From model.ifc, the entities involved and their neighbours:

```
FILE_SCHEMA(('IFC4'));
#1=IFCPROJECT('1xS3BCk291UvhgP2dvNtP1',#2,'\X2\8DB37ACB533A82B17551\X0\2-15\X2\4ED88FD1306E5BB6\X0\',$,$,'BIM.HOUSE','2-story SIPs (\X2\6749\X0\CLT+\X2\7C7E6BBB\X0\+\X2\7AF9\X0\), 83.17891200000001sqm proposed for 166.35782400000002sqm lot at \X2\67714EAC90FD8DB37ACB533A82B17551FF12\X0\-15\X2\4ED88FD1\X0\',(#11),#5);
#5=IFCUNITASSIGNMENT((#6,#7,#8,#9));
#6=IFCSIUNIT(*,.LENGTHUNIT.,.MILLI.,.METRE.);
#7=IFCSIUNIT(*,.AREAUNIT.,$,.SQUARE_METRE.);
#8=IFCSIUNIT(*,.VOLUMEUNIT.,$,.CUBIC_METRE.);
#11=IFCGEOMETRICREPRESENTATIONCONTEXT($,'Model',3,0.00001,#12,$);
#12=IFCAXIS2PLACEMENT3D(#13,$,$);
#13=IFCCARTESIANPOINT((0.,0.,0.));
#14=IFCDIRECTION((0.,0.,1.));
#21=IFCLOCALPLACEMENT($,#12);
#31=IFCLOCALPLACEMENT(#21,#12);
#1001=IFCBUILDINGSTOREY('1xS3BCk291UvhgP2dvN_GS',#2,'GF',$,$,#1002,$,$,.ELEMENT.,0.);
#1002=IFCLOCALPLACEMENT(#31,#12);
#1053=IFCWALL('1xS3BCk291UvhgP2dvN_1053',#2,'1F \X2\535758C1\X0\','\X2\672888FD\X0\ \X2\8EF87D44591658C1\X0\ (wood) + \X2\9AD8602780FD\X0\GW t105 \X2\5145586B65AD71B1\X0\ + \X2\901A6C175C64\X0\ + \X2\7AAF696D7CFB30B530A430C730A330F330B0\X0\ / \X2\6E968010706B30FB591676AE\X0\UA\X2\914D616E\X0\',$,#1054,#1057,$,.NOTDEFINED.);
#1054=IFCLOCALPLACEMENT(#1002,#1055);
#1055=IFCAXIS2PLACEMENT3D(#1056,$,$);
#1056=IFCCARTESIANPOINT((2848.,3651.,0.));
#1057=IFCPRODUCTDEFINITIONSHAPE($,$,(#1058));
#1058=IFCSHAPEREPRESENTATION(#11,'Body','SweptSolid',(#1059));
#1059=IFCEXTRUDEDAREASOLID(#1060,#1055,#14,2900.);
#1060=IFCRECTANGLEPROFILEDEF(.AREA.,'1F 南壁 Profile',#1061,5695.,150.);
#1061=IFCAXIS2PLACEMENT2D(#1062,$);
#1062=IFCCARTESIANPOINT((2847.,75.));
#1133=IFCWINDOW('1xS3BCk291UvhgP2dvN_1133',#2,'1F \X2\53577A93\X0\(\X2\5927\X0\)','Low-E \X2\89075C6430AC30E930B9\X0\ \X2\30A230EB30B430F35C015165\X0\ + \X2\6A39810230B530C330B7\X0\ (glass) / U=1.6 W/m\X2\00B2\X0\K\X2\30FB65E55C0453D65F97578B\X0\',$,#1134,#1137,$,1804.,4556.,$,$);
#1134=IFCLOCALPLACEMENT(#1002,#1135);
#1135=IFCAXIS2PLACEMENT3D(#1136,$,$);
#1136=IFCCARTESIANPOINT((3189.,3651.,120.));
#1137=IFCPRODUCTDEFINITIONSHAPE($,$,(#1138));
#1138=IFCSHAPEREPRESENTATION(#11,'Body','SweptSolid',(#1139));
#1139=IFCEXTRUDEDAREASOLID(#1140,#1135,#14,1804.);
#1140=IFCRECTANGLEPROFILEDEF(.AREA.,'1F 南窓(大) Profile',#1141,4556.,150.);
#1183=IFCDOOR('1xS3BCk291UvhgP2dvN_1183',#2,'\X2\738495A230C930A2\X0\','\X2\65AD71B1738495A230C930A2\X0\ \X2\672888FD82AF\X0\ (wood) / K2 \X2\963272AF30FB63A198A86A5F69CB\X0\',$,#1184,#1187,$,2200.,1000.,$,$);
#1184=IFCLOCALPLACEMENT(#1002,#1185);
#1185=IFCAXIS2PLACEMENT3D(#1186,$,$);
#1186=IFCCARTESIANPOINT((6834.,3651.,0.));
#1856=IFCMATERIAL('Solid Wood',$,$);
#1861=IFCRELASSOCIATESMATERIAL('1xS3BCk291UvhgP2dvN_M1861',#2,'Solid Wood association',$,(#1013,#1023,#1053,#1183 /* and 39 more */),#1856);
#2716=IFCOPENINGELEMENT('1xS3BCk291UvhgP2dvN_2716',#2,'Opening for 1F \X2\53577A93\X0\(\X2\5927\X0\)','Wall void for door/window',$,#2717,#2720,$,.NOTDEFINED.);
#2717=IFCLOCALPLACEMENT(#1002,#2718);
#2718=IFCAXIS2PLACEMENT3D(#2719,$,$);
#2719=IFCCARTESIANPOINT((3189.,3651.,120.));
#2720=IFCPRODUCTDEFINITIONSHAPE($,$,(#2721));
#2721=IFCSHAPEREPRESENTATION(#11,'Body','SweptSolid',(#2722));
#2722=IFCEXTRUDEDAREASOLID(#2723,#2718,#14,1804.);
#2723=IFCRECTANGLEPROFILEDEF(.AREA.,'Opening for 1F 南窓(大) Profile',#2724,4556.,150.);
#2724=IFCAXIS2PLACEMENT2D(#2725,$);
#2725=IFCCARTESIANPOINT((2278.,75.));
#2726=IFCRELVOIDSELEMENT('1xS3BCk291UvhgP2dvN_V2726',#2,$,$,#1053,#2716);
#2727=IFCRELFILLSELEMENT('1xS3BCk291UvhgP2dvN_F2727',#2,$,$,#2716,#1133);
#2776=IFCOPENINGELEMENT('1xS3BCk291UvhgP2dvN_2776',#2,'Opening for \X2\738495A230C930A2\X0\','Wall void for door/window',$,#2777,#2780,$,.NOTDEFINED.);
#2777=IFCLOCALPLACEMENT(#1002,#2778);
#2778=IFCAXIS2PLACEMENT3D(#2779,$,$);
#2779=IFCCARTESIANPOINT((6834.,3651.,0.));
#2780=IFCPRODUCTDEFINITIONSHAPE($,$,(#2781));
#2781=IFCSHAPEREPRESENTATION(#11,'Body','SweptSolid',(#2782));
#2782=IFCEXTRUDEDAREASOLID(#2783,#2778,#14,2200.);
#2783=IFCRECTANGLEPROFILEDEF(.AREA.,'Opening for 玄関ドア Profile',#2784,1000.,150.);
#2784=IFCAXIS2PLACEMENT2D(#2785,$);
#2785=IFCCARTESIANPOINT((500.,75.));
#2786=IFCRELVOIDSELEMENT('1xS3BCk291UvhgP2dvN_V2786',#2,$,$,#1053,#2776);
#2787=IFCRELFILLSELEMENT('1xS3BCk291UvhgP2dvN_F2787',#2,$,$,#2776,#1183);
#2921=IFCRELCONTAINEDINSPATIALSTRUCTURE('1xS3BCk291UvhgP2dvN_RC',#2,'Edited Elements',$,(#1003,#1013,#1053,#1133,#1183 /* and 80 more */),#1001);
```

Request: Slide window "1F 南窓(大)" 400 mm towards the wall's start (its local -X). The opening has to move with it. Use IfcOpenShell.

```python
import ifcopenshell
import ifcopenshell.api.geometry
import ifcopenshell.util.placement

model = ifcopenshell.open("model.ifc")

window = model.by_guid("1xS3BCk291UvhgP2dvN_1133")
opening = window.FillsVoids[0].RelatingOpeningElement
wall = opening.VoidsElements[0].RelatingBuildingElement

wall_matrix = ifcopenshell.util.placement.get_local_placement(wall.ObjectPlacement)
shift = wall_matrix[:3, 0] * -400.0
before = ifcopenshell.util.placement.get_local_placement(window.ObjectPlacement)[:3, 3].copy()

# The window is not placed relative to its opening, so move both.
for product in (opening, window):
    matrix = ifcopenshell.util.placement.get_local_placement(product.ObjectPlacement)
    matrix[:3, 3] += shift
    ifcopenshell.api.geometry.edit_object_placement(model, product=product, matrix=matrix, is_si=False)

after = ifcopenshell.util.placement.get_local_placement(window.ObjectPlacement)[:3, 3]
print("window moved by", (after - before).round(3) + 0.0)

model.write("model_edited.ifc")
```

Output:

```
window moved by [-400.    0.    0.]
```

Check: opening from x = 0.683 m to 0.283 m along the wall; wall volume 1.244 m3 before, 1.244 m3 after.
